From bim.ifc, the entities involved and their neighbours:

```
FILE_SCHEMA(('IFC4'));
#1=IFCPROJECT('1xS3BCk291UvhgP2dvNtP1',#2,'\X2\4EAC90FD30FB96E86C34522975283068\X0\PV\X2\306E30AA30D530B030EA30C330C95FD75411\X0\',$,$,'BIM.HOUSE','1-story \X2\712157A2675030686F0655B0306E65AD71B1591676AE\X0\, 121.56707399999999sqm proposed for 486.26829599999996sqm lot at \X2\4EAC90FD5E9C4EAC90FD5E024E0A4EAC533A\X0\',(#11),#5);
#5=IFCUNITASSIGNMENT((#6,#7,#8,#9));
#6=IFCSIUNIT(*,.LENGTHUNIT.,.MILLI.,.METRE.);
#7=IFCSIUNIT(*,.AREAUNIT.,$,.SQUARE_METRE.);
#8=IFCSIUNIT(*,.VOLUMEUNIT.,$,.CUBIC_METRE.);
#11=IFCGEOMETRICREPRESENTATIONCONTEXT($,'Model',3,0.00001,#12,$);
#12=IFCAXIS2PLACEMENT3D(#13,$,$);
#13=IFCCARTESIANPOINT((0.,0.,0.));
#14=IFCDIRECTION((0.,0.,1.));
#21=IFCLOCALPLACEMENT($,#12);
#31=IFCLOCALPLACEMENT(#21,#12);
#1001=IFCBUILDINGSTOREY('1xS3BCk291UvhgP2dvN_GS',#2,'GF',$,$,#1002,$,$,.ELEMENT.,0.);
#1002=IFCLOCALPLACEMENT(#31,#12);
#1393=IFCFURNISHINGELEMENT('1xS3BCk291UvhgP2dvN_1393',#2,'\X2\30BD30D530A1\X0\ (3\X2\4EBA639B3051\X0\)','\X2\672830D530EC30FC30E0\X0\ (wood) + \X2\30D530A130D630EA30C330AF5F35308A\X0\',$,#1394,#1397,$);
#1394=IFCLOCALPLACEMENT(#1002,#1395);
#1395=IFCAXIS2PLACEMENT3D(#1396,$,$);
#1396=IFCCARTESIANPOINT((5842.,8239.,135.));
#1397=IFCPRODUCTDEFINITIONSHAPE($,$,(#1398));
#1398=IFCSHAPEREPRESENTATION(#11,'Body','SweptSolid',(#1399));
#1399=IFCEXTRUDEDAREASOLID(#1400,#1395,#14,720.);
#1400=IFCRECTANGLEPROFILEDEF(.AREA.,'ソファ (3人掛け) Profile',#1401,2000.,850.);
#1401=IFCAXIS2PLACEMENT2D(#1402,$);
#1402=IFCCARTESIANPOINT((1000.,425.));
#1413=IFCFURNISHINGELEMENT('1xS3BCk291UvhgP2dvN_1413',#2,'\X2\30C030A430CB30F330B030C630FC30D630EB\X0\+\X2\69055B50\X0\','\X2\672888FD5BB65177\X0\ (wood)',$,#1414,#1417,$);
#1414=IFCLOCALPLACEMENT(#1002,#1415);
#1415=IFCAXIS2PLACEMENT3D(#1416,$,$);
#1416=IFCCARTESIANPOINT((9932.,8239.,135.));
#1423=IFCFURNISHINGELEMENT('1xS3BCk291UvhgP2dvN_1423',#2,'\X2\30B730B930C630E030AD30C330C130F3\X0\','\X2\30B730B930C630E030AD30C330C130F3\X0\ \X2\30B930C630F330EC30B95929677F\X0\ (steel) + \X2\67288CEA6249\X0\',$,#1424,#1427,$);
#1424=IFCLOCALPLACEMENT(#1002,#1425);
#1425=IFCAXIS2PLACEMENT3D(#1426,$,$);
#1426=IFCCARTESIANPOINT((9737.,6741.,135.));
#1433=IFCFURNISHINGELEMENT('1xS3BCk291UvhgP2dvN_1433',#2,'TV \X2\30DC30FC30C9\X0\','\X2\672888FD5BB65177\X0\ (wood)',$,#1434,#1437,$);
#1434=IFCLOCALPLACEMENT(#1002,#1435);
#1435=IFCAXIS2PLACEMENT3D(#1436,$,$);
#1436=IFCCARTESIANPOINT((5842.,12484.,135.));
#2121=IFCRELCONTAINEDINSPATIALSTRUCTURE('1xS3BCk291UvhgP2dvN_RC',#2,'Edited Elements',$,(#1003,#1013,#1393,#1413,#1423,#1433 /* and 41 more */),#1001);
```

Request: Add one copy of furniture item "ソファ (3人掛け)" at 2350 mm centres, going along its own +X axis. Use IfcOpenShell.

```python
import ifcopenshell
import ifcopenshell.api.geometry
import ifcopenshell.api.root
import ifcopenshell.util.element
import ifcopenshell.util.placement

model = ifcopenshell.open("bim.ifc")


def reuse_history(source, copy):
    """copy_class also copies each property set's owner history, people and application; keep the originals."""
    for rel in copy.IsDefinedBy:
        if rel.is_a("IfcRelDefinesByProperties") and (history := rel.RelatingPropertyDefinition.OwnerHistory):
            rel.RelatingPropertyDefinition.OwnerHistory = source.OwnerHistory
            ifcopenshell.util.element.remove_deep2(model, history)


source = model.by_guid("1xS3BCk291UvhgP2dvN_1393")
base = ifcopenshell.util.placement.get_local_placement(source.ObjectPlacement)
step = base[:3, 0] * 2350.0

for i in range(1, 2):
    copy = ifcopenshell.api.root.copy_class(model, product=source)
    copy.Representation = ifcopenshell.util.element.copy_deep(
        model, source.Representation, exclude=["IfcGeometricRepresentationContext", "IfcRepresentationMap"]
    )
    reuse_history(source, copy)
    matrix = base.copy()
    matrix[:3, 3] += i * step
    print("added at", matrix[:3, 3].round(3) + 0.0)
    ifcopenshell.api.geometry.edit_object_placement(model, product=copy, matrix=matrix, is_si=False)

model.write("bim_rev.ifc")
```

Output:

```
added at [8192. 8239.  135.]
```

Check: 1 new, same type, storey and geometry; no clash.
